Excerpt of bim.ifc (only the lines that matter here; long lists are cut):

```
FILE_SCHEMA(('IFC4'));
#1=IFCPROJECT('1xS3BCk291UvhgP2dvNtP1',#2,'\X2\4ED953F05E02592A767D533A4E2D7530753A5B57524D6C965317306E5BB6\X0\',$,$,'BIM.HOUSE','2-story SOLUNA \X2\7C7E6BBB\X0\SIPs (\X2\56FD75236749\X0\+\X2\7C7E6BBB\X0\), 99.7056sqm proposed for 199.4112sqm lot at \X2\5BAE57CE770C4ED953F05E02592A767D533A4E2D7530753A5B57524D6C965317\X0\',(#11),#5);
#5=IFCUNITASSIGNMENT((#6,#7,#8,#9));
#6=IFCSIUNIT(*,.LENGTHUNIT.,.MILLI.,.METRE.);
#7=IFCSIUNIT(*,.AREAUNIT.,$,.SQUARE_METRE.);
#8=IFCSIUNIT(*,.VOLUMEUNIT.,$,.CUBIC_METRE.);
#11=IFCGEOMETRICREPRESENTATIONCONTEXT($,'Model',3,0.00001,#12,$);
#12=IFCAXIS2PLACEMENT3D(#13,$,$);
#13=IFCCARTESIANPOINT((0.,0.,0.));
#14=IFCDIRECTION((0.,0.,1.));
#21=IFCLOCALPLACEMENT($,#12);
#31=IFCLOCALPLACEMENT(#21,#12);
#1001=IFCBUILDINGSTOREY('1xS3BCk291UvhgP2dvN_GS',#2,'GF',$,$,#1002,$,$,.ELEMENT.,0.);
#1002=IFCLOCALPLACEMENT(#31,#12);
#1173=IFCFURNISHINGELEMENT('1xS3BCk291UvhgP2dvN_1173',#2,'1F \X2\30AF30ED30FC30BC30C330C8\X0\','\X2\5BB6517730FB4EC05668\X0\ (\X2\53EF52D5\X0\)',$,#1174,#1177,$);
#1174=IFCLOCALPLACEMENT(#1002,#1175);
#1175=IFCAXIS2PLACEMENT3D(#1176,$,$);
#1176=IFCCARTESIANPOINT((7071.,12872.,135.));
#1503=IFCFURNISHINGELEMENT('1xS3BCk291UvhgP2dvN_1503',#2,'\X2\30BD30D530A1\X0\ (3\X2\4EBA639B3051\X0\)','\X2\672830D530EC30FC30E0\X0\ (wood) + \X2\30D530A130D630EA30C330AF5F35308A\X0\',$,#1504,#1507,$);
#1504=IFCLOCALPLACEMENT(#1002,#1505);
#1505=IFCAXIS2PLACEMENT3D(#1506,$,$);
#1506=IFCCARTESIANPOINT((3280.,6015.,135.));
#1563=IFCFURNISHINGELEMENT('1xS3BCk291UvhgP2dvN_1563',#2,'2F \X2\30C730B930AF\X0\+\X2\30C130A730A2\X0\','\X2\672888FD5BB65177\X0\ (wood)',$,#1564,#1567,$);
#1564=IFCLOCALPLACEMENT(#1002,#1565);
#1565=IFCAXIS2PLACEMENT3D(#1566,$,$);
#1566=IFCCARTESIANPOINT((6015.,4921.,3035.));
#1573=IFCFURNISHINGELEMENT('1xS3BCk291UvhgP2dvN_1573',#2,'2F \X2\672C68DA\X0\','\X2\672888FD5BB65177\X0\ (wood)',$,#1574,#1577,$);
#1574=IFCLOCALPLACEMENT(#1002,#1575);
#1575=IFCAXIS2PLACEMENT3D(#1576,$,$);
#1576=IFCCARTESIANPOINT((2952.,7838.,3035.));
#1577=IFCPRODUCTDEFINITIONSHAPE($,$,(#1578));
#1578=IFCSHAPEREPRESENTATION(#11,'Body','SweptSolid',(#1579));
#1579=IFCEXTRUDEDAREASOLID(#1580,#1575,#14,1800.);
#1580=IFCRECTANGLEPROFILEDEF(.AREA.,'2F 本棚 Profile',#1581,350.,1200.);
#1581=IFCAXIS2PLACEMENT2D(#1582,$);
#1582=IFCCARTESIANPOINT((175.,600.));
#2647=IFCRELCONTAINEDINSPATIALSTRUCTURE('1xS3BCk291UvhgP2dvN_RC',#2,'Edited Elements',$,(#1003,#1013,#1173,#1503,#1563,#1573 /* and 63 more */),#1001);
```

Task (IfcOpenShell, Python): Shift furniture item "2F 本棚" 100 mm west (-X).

```python
import ifcopenshell
import ifcopenshell.api.geometry
import ifcopenshell.util.placement
import ifcopenshell.util.unit

model = ifcopenshell.open("bim.ifc")
unit_scale = ifcopenshell.util.unit.calculate_unit_scale(model)

item = model.by_id(1573)
matrix = ifcopenshell.util.placement.get_local_placement(item.ObjectPlacement)
matrix[0, 3] -= 0.1 / unit_scale
ifcopenshell.api.geometry.edit_object_placement(model, product=item, matrix=matrix, is_si=False)

print(ifcopenshell.util.placement.get_local_placement(item.ObjectPlacement).round(3) + 0.0)

model.write("bim_v2.ifc")
```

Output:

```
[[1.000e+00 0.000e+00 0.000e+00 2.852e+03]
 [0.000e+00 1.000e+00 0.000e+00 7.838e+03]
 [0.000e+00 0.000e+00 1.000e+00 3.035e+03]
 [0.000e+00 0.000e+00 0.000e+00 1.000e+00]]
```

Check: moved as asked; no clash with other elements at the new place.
